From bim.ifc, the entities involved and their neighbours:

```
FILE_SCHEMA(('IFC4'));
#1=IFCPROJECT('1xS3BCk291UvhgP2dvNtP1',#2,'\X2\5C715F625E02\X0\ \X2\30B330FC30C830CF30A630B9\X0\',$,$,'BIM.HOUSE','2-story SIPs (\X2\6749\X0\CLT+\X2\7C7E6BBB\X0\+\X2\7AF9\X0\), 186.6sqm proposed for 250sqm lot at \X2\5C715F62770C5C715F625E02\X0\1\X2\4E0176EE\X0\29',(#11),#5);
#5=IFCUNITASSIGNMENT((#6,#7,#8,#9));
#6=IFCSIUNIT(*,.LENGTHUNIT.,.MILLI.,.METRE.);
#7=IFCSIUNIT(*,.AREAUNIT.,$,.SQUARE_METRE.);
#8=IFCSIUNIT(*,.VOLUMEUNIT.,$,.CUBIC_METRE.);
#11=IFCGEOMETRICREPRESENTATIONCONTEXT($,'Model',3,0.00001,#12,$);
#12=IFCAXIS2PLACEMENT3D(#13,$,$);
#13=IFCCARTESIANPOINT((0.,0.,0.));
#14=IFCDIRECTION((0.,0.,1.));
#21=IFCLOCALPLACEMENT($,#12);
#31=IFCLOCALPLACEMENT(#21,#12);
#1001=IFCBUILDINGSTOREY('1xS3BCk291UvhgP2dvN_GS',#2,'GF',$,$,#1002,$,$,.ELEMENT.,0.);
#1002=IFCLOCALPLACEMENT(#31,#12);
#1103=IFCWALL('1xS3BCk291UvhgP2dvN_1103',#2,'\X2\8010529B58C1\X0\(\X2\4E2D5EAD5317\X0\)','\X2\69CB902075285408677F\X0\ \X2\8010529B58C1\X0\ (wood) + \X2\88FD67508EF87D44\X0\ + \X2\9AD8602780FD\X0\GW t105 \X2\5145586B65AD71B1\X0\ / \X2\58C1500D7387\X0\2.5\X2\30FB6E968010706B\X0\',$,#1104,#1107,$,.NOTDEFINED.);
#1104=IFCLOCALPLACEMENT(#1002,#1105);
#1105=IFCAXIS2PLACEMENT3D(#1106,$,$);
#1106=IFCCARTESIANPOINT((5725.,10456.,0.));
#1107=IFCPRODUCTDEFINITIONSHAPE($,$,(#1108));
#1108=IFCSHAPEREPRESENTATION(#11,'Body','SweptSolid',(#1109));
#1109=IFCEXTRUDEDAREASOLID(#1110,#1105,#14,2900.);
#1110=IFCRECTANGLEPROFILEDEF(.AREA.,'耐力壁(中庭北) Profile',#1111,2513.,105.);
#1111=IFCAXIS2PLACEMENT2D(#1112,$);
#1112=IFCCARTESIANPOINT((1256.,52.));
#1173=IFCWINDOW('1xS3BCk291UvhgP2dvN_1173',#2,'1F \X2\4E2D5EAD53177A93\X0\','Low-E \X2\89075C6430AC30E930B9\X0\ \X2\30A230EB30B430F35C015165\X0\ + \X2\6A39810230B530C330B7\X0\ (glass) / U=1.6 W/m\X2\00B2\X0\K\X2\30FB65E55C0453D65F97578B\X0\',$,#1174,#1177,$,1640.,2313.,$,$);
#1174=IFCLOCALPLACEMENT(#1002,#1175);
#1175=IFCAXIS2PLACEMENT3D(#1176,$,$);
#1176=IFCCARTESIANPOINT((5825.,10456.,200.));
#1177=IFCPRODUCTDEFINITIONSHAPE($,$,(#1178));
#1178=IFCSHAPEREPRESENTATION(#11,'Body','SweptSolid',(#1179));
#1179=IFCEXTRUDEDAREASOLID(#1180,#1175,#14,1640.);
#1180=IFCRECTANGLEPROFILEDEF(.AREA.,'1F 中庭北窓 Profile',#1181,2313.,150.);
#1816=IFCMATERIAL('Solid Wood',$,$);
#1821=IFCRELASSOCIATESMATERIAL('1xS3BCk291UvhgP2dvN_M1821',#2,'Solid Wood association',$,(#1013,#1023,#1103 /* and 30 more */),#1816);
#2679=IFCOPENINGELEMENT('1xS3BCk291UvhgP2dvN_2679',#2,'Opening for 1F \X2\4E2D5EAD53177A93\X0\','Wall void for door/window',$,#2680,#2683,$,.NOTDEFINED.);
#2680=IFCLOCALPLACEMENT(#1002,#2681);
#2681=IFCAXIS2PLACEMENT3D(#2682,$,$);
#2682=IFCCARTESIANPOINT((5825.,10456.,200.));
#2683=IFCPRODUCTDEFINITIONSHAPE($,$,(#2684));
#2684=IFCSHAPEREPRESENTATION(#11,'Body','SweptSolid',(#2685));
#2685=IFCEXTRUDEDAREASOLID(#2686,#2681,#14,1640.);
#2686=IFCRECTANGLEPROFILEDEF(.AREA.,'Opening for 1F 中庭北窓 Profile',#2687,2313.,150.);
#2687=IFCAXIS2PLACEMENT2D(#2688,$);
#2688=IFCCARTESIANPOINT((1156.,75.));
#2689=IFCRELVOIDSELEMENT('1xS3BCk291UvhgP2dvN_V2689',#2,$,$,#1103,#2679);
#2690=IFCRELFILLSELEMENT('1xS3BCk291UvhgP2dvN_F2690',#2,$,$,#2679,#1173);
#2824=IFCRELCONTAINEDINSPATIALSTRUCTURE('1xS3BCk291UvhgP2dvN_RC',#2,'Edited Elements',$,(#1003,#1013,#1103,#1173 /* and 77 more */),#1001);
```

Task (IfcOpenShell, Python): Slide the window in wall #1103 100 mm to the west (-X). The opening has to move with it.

```python
import ifcopenshell
import ifcopenshell.api.geometry
import ifcopenshell.util.placement

model = ifcopenshell.open("bim.ifc")

window = model.by_id(1173)
opening = window.FillsVoids[0].RelatingOpeningElement
wall = opening.VoidsElements[0].RelatingBuildingElement

wall_matrix = ifcopenshell.util.placement.get_local_placement(wall.ObjectPlacement)
shift = wall_matrix[:3, 0] * -100.0
before = ifcopenshell.util.placement.get_local_placement(window.ObjectPlacement)[:3, 3].copy()

# The window is not placed relative to its opening, so move both.
for product in (opening, window):
    matrix = ifcopenshell.util.placement.get_local_placement(product.ObjectPlacement)
    matrix[:3, 3] += shift
    ifcopenshell.api.geometry.edit_object_placement(model, product=product, matrix=matrix, is_si=False)

after = ifcopenshell.util.placement.get_local_placement(window.ObjectPlacement)[:3, 3]
print("window moved by", (after - before).round(3) + 0.0)

model.write("bim_v2.ifc")
```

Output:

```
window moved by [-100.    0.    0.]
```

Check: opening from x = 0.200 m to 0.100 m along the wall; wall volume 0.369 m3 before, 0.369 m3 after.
